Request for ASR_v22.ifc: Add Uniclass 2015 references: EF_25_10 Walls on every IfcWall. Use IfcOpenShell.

First a look at what the model holds.

```python
import ifcopenshell

model = ifcopenshell.open("ASR_v22.ifc")
print(model.schema)
print("classifications:", [c.Name for c in model.by_type("IfcClassification")])
for ifc_class in ("IfcDoor", "IfcRoof", "IfcStair", "IfcWall", "IfcWindow"):
    print(ifc_class, len(model.by_type(ifc_class)))
```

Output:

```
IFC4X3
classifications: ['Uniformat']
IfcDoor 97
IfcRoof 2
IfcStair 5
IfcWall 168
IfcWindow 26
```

```python
import ifcopenshell
import ifcopenshell.api.classification

model = ifcopenshell.open("ASR_v22.ifc")

system = ifcopenshell.api.classification.add_classification(model, classification="Uniclass 2015")

codes = {
    "IfcWall": ("EF_25_10", "Walls"),
}
for ifc_class, (code, name) in codes.items():
    products = model.by_type(ifc_class)
    ifcopenshell.api.classification.add_reference(
        model, products=products, classification=system, identification=code, name=name
    )
    print(code, len(products))

model.write("ASR_v22_v2.ifc")
```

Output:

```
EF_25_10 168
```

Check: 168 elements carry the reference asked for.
